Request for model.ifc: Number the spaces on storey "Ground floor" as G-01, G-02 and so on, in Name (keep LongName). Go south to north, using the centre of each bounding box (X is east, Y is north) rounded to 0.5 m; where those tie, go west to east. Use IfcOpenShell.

First a look at what the model holds.

```python
import ifcopenshell
import ifcopenshell.util.element
import ifcopenshell.util.placement

model = ifcopenshell.open("model.ifc")
print(model.schema)
storey = next(s for s in model.by_type("IfcBuildingStorey") if s.Name == "Ground floor")
spaces = [e for e in ifcopenshell.util.element.get_decomposition(storey) if e.is_a("IfcSpace")]
for e in sorted(spaces, key=lambda e: e.id()):
    origin = ifcopenshell.util.placement.get_local_placement(e.ObjectPlacement)[:3, 3]
    print(e.id(), e.Name, e.LongName, origin.round(2) + 0.0, sep=" | ")
```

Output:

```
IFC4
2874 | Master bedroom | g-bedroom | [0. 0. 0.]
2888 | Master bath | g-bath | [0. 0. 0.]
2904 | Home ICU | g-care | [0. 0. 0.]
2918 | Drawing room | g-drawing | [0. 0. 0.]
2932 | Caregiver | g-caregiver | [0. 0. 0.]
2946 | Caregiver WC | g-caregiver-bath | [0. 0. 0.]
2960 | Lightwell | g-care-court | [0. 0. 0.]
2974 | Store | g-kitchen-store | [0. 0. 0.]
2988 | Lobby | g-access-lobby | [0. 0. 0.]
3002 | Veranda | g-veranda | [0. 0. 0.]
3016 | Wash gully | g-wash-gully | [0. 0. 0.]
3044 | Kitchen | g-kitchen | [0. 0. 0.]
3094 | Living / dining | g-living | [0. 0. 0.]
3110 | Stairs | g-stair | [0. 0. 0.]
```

```python
import ifcopenshell
import ifcopenshell.geom
import ifcopenshell.util.element
import ifcopenshell.util.shape

model = ifcopenshell.open("model.ifc")
settings = ifcopenshell.geom.settings()
settings.set("use-world-coords", True)


def centre(element):
    shape = ifcopenshell.geom.create_shape(settings, element)
    return ifcopenshell.util.shape.get_bbox_centroid(shape.geometry)


storey = next(s for s in model.by_type("IfcBuildingStorey") if s.Name == "Ground floor")
spaces = [e for e in ifcopenshell.util.element.get_decomposition(storey) if e.is_a("IfcSpace")]

# Insertion points can sit at a corner or the storey origin, so sort by the geometry (in metres).
centres = {e: centre(e) for e in spaces}
spaces.sort(key=lambda e: (round(centres[e][1] / 0.5), centres[e][0]))

for i, e in enumerate(spaces, start=1):
    number = f"G-{i:02d}"
    e.Name = number
    print(e.id(), number)

model.write("model_v2.ifc")
```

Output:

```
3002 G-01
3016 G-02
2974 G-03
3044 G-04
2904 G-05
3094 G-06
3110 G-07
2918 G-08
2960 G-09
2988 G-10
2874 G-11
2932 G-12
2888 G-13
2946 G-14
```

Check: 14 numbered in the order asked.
